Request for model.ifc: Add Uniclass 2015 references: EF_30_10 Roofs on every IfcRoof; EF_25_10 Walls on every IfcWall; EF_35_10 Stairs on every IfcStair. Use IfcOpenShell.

First a look at what the model holds.

```python
import ifcopenshell

model = ifcopenshell.open("model.ifc")
print(model.schema)
print("classifications:", [c.Name for c in model.by_type("IfcClassification")])
for ifc_class in ("IfcDoor", "IfcRoof", "IfcStair", "IfcWall", "IfcWindow"):
    print(ifc_class, len(model.by_type(ifc_class)))
```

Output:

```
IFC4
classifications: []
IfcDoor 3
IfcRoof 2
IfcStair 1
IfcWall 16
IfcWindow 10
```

```python
import ifcopenshell
import ifcopenshell.api.classification

model = ifcopenshell.open("model.ifc")

system = ifcopenshell.api.classification.add_classification(model, classification="Uniclass 2015")

codes = {
    "IfcRoof": ("EF_30_10", "Roofs"),
    "IfcWall": ("EF_25_10", "Walls"),
    "IfcStair": ("EF_35_10", "Stairs"),
}
for ifc_class, (code, name) in codes.items():
    products = model.by_type(ifc_class)
    ifcopenshell.api.classification.add_reference(
        model, products=products, classification=system, identification=code, name=name
    )
    print(code, len(products))

model.write("model_updated.ifc")
```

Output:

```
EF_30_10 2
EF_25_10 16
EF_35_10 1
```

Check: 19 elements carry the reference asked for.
